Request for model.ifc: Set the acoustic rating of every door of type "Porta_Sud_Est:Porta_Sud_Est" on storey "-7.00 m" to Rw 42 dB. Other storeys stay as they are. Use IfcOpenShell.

First a look at what the model holds.

```python
import ifcopenshell
import ifcopenshell.util.element

model = ifcopenshell.open("model.ifc")
print(model.schema)
storey = next(s for s in model.by_type("IfcBuildingStorey") if s.Name == "-7.00 m")
doors = [e for e in ifcopenshell.util.element.get_decomposition(storey) if e.is_a("IfcDoor")]
seen = {}
for e in doors:
    element_type = ifcopenshell.util.element.get_type(e)
    key = (element_type.Name if element_type != e and element_type else None, ifcopenshell.util.element.get_pset(e, "Pset_DoorCommon", "AcousticRating"))
    seen[key] = seen.get(key, 0) + 1
for (name, value), count in sorted(seen.items(), key=str):
    print(count, "x", name, "|", value)
```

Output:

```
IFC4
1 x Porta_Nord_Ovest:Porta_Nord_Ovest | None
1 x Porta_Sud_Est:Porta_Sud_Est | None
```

```python
import ifcopenshell
import ifcopenshell.api.pset
import ifcopenshell.util.element

model = ifcopenshell.open("model.ifc")

storey = next(s for s in model.by_type("IfcBuildingStorey") if s.Name == "-7.00 m")
doors = [e for e in ifcopenshell.util.element.get_decomposition(storey) if e.is_a("IfcDoor")]

count = 0
for e in doors:
    element_type = ifcopenshell.util.element.get_type(e)
    if element_type in (None, e) or element_type.Name != "Porta_Sud_Est:Porta_Sud_Est":
        continue
    # add_pset returns the element's existing set when there is one.
    pset = ifcopenshell.api.pset.add_pset(model, product=e, name="Pset_DoorCommon")
    ifcopenshell.api.pset.edit_pset(model, pset=pset, properties={"AcousticRating": "Rw 42 dB"})
    count += 1

print(count, "doors updated")

model.write("model_updated.ifc")
```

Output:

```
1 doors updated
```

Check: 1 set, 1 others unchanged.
